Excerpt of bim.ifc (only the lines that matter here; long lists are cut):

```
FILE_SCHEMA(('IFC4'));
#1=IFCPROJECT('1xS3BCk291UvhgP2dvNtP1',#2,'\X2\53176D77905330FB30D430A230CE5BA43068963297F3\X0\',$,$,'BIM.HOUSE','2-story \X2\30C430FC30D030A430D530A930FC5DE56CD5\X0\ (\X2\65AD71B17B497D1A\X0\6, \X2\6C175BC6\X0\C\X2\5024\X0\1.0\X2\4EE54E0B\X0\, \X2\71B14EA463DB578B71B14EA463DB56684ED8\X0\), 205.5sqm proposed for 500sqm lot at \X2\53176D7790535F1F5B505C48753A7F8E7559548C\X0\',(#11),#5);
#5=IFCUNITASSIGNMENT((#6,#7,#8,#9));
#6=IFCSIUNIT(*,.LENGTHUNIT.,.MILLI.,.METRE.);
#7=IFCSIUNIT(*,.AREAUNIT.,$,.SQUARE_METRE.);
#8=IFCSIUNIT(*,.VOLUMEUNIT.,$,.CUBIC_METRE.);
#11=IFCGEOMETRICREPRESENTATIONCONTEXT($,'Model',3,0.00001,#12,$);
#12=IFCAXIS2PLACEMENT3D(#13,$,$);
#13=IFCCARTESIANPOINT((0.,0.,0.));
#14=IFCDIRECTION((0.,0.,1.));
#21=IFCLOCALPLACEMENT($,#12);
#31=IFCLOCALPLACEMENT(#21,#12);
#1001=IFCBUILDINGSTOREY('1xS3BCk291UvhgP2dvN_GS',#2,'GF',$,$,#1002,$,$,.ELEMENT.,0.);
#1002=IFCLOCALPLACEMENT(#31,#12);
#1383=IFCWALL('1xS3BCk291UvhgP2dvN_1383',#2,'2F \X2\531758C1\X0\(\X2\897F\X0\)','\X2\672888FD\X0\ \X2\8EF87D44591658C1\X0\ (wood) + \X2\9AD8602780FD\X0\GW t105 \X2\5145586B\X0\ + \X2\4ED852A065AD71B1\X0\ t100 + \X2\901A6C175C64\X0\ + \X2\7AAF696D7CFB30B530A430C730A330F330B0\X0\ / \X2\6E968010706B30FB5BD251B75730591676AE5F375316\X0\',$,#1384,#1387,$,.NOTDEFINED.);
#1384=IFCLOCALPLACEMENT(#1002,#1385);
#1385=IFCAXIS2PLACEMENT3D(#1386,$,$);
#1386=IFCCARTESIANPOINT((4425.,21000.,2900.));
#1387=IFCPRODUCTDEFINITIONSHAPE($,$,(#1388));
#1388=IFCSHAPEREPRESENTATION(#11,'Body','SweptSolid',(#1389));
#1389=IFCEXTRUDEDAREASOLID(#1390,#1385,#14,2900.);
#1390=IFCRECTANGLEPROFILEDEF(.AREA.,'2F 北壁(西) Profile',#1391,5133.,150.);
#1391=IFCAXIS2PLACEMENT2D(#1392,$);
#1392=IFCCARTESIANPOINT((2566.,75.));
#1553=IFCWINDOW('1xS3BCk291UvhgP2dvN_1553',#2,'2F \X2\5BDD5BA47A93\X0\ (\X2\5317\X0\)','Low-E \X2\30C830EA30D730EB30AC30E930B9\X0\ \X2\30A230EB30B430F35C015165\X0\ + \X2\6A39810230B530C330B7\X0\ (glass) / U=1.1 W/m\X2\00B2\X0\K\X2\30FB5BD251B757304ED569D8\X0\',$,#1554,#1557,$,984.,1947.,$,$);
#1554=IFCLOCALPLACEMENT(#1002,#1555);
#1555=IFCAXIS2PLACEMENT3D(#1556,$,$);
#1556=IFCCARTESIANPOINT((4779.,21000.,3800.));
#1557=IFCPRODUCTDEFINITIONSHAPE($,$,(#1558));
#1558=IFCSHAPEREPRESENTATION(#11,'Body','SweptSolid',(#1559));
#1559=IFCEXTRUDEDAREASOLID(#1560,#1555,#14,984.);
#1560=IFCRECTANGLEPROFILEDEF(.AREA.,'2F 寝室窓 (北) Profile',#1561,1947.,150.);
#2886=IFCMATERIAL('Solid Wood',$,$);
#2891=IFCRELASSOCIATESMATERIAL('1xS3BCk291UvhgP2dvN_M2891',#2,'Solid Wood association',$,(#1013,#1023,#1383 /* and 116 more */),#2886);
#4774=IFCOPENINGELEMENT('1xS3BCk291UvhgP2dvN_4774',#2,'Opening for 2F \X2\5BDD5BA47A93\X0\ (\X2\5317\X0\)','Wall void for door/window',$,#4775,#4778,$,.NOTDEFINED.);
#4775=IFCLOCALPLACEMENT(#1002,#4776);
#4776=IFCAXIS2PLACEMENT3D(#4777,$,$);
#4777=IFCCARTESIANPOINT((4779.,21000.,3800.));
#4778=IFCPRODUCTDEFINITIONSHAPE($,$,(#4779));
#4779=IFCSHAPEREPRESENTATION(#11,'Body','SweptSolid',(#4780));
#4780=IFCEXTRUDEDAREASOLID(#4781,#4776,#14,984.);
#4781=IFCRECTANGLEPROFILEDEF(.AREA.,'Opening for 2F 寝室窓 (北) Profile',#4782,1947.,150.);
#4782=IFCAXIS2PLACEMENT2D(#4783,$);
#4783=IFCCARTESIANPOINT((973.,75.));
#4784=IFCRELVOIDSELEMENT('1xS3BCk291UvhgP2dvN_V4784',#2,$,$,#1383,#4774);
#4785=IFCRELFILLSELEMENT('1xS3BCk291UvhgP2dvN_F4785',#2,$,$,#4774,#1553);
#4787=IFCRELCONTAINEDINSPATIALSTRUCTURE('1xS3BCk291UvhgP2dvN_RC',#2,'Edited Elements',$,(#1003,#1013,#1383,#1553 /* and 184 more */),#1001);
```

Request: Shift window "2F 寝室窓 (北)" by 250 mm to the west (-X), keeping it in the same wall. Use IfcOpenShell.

```python
import ifcopenshell
import ifcopenshell.api.geometry
import ifcopenshell.util.placement
import ifcopenshell.util.unit

model = ifcopenshell.open("bim.ifc")
unit_scale = ifcopenshell.util.unit.calculate_unit_scale(model)

window = model.by_id(1553)
opening = window.FillsVoids[0].RelatingOpeningElement
wall = opening.VoidsElements[0].RelatingBuildingElement

wall_matrix = ifcopenshell.util.placement.get_local_placement(wall.ObjectPlacement)
shift = wall_matrix[:3, 0] * -0.25 / unit_scale
before = ifcopenshell.util.placement.get_local_placement(window.ObjectPlacement)[:3, 3].copy()

# The window is not placed relative to its opening, so move both.
for product in (opening, window):
    matrix = ifcopenshell.util.placement.get_local_placement(product.ObjectPlacement)
    matrix[:3, 3] += shift
    ifcopenshell.api.geometry.edit_object_placement(model, product=product, matrix=matrix, is_si=False)

after = ifcopenshell.util.placement.get_local_placement(window.ObjectPlacement)[:3, 3]
print("window moved by", (after - before).round(3) + 0.0)

model.write("bim_rev.ifc")
```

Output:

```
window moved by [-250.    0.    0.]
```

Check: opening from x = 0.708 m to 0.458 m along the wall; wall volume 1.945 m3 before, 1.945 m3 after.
